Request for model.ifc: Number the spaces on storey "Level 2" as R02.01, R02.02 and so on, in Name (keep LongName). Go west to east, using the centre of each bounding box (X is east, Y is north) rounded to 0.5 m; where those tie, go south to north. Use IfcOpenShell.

First a look at what the model holds.

```python
import ifcopenshell
import ifcopenshell.util.element
import ifcopenshell.util.placement

model = ifcopenshell.open("model.ifc")
print(model.schema)
storey = next(s for s in model.by_type("IfcBuildingStorey") if s.Name == "Level 2")
spaces = [e for e in ifcopenshell.util.element.get_decomposition(storey) if e.is_a("IfcSpace")]
for e in sorted(spaces, key=lambda e: e.id()):
    origin = ifcopenshell.util.placement.get_local_placement(e.ObjectPlacement)[:3, 3]
    print(e.id(), e.Name, e.LongName, origin.round(2) + 0.0, sep=" | ")
```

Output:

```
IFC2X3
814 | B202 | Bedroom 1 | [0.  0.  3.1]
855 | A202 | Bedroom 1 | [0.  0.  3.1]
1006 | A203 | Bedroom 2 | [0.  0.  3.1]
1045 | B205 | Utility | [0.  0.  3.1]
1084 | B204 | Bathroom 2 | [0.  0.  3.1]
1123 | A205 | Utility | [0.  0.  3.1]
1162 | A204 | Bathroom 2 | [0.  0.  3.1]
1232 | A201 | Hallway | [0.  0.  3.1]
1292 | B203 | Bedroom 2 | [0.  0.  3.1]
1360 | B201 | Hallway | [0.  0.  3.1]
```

```python
import ifcopenshell
import ifcopenshell.geom
import ifcopenshell.util.element
import ifcopenshell.util.shape

model = ifcopenshell.open("model.ifc")
settings = ifcopenshell.geom.settings()
settings.set("use-world-coords", True)


def centre(element):
    shape = ifcopenshell.geom.create_shape(settings, element)
    return ifcopenshell.util.shape.get_bbox_centroid(shape.geometry)


storey = next(s for s in model.by_type("IfcBuildingStorey") if s.Name == "Level 2")
spaces = [e for e in ifcopenshell.util.element.get_decomposition(storey) if e.is_a("IfcSpace")]

# Insertion points can sit at a corner or the storey origin, so sort by the geometry (in metres).
centres = {e: centre(e) for e in spaces}
spaces.sort(key=lambda e: (round(centres[e][0] / 0.5), centres[e][1]))

for i, e in enumerate(spaces, start=1):
    number = f"R02.{i:02d}"
    e.Name = number
    print(e.id(), number)

model.write("model_rev.ifc")
```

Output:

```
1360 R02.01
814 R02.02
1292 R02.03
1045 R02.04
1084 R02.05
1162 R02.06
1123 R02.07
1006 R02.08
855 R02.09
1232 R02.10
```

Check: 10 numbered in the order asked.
